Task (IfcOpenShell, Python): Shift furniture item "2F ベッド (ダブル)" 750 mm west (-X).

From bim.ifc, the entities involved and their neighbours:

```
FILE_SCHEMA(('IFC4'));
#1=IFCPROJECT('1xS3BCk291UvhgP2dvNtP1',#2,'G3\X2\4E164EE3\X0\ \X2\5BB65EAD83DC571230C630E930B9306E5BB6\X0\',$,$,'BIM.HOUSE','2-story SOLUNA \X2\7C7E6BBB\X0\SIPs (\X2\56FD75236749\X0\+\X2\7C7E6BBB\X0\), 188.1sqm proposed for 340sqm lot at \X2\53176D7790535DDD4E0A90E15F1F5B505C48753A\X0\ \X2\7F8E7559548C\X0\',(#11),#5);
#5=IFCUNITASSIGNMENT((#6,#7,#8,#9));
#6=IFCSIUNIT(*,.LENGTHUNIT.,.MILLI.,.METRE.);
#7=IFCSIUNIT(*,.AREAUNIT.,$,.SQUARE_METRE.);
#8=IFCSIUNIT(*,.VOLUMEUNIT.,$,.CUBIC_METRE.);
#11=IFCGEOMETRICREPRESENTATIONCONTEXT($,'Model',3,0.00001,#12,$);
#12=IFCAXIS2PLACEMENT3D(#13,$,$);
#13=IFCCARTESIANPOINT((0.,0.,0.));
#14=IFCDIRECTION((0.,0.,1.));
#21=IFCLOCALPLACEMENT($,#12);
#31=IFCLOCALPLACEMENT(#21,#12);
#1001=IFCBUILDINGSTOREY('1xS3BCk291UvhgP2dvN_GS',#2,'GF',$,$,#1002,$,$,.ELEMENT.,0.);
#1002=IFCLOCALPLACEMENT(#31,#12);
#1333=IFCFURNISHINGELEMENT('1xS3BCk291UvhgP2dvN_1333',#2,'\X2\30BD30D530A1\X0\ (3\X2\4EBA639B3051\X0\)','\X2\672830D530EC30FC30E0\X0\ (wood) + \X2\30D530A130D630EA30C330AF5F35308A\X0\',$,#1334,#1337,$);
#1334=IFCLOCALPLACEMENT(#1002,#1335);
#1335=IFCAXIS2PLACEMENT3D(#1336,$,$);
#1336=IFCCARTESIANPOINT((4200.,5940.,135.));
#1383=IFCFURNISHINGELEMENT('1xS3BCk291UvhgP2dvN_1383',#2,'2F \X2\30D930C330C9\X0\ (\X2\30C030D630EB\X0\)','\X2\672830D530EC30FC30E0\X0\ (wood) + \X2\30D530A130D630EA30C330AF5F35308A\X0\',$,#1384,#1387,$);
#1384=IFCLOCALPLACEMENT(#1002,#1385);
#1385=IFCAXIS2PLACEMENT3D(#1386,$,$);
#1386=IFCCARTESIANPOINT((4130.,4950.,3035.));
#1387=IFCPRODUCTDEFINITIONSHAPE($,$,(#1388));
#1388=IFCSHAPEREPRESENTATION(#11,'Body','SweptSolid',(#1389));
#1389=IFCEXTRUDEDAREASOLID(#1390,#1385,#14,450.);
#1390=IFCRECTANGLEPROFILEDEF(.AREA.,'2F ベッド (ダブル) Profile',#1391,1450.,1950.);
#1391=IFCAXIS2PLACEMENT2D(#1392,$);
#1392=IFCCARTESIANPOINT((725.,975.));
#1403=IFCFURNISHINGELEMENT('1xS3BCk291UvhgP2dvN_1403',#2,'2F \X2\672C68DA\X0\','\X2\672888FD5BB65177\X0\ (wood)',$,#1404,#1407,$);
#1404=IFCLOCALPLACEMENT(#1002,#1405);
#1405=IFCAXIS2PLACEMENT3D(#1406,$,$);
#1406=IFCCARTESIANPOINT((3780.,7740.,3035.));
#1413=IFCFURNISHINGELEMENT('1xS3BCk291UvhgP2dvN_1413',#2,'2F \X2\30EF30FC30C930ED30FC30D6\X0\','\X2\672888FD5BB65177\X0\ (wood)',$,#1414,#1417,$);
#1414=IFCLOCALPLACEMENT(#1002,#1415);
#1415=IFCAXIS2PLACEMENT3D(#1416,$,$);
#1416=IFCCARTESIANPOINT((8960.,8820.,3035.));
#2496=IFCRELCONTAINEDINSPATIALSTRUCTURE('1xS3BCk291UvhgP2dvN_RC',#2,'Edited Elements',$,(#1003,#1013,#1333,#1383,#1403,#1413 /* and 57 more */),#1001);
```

```python
import ifcopenshell
import ifcopenshell.api.geometry
import ifcopenshell.util.placement

model = ifcopenshell.open("bim.ifc")

item = model.by_guid("1xS3BCk291UvhgP2dvN_1383")
matrix = ifcopenshell.util.placement.get_local_placement(item.ObjectPlacement)
matrix[0, 3] -= 750.0
ifcopenshell.api.geometry.edit_object_placement(model, product=item, matrix=matrix, is_si=False)

print(ifcopenshell.util.placement.get_local_placement(item.ObjectPlacement).round(3) + 0.0)

model.write("bim_v2.ifc")
```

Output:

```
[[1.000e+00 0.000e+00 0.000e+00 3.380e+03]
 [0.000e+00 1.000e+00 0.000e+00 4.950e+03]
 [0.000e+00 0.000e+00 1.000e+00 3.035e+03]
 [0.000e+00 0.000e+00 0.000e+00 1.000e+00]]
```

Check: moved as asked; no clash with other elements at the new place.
